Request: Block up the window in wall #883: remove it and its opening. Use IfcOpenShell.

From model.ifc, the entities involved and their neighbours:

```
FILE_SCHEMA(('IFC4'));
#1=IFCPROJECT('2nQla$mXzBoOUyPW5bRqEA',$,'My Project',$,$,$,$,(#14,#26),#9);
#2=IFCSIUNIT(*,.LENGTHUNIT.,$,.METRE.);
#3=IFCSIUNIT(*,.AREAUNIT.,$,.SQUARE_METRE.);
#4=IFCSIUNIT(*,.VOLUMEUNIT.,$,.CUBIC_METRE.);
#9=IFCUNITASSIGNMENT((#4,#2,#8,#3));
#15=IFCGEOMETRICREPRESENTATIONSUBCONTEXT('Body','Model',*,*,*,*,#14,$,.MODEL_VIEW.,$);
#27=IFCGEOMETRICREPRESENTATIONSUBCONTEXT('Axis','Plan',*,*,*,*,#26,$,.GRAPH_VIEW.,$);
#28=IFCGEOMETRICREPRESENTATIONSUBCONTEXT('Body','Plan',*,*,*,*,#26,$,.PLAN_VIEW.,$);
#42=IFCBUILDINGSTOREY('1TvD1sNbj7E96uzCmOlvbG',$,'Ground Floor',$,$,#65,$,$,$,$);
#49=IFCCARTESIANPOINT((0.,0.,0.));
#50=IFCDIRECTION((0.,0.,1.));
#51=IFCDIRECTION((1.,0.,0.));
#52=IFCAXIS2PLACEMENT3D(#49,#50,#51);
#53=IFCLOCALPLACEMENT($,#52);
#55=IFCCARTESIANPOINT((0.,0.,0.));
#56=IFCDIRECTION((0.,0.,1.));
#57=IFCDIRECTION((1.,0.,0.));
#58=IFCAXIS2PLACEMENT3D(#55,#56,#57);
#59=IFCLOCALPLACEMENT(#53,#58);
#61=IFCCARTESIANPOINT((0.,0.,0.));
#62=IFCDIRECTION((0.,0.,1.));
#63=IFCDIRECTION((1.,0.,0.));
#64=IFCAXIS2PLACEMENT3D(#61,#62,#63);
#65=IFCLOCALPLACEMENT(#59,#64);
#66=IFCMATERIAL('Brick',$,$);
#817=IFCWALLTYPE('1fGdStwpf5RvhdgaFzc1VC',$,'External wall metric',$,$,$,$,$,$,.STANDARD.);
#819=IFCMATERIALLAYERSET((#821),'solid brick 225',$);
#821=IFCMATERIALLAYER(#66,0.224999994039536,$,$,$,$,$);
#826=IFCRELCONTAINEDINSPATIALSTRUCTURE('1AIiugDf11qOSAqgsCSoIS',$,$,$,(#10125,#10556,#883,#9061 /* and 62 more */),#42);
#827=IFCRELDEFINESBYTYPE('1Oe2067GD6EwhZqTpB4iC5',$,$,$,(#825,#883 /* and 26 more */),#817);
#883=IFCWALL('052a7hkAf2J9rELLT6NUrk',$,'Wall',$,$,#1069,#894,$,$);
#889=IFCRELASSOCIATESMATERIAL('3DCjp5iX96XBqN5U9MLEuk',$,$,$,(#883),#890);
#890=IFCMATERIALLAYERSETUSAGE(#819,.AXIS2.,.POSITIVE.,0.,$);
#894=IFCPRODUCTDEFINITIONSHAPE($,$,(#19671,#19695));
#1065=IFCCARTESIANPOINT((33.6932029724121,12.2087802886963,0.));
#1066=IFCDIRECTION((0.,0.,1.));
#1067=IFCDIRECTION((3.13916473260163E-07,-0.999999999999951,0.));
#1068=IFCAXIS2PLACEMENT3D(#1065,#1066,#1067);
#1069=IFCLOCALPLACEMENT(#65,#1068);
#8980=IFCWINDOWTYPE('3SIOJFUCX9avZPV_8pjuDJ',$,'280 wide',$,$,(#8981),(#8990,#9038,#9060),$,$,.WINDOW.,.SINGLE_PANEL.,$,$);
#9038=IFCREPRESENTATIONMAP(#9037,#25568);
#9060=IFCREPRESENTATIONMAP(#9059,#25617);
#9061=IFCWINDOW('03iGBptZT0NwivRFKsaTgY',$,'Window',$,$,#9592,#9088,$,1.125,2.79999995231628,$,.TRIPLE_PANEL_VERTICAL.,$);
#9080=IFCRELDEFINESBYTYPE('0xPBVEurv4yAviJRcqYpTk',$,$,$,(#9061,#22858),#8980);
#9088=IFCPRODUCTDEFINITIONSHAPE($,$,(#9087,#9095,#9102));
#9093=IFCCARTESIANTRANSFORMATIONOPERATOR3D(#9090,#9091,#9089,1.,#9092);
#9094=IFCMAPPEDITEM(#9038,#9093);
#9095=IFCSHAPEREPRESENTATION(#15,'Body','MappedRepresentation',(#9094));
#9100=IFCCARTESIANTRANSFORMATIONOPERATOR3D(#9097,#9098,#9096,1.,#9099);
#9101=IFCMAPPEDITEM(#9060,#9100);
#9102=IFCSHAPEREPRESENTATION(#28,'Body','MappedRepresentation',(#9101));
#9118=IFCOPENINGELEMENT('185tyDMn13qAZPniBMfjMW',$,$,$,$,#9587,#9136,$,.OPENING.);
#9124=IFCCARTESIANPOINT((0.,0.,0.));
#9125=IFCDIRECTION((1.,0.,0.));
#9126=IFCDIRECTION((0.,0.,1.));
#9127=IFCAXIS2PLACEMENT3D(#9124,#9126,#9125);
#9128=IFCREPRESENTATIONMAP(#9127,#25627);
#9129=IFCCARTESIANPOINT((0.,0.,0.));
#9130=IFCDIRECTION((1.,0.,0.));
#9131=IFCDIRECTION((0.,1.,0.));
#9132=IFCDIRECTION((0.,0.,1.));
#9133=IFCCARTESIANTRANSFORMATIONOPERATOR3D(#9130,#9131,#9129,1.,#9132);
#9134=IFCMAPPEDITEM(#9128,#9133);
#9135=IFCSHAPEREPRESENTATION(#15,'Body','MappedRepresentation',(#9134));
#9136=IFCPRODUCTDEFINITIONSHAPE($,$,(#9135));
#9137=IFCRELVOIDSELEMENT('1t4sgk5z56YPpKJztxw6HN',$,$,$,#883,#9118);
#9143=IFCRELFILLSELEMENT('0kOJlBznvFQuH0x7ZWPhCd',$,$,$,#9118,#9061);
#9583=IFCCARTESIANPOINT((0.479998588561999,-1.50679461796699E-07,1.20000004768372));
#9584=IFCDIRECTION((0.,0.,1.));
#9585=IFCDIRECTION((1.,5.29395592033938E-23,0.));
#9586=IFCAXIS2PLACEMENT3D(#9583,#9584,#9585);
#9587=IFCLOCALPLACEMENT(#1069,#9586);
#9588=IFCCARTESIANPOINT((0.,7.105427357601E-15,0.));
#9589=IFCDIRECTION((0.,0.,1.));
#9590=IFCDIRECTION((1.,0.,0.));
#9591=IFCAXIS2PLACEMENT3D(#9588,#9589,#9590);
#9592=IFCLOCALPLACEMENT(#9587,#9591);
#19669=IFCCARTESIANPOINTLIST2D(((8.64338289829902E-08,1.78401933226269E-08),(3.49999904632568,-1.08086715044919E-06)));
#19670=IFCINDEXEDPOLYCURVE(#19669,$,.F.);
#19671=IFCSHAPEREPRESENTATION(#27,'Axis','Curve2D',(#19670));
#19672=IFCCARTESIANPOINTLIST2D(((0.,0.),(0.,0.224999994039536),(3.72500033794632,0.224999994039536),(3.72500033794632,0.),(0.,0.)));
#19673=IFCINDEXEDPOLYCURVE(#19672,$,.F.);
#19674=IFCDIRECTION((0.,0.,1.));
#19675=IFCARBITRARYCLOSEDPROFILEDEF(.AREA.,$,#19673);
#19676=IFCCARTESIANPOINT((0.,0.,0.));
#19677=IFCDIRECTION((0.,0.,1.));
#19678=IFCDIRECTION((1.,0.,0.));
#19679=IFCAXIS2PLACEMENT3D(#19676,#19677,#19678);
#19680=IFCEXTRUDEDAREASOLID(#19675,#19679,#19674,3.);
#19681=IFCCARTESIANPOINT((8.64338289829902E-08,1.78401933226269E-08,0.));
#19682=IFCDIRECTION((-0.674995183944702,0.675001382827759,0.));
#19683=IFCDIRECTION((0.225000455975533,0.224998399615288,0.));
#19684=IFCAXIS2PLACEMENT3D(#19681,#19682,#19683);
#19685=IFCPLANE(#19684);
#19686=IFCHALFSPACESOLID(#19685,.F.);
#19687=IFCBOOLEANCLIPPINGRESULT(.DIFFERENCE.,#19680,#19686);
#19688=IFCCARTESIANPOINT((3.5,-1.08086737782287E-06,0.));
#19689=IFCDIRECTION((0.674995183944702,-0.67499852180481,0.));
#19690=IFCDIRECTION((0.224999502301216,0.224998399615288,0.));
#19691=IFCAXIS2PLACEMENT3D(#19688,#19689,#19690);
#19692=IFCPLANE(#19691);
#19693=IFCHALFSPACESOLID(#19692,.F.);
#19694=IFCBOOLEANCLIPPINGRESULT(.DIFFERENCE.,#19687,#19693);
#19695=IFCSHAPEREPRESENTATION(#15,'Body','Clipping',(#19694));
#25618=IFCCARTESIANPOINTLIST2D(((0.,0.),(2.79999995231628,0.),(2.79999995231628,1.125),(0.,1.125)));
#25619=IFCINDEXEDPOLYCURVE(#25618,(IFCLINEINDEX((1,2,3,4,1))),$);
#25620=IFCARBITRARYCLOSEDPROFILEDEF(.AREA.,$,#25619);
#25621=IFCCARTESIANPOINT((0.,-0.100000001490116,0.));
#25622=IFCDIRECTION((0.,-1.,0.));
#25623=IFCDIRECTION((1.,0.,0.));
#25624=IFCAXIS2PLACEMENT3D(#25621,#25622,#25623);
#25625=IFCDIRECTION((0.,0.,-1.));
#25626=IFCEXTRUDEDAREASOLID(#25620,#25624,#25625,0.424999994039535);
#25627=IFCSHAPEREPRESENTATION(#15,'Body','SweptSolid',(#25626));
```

```python
import ifcopenshell
import ifcopenshell.api.feature
import ifcopenshell.api.root
import ifcopenshell.geom
import ifcopenshell.util.shape

model = ifcopenshell.open("model.ifc")
settings = ifcopenshell.geom.settings()


def volume(element):
    """Net volume in cubic metres, openings subtracted."""
    shape = ifcopenshell.geom.create_shape(settings, element)
    return ifcopenshell.util.shape.get_volume(shape.geometry)


window = model.by_id(9061)
opening = window.FillsVoids[0].RelatingOpeningElement
wall = opening.VoidsElements[0].RelatingBuildingElement
before = volume(wall)

ifcopenshell.api.root.remove_product(model, product=window)
ifcopenshell.api.feature.remove_feature(model, feature=opening)

after = volume(wall)

print(f"wall volume {before:.3f} -> {after:.3f} m3")

model.write("model_v2.ifc")
```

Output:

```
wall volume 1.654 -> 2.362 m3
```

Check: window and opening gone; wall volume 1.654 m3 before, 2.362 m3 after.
